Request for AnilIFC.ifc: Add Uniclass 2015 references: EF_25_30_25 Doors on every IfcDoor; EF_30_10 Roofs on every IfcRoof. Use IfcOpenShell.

First a look at what the model holds.

```python
import ifcopenshell

model = ifcopenshell.open("AnilIFC.ifc")
print(model.schema)
print("classifications:", [c.Name for c in model.by_type("IfcClassification")])
for ifc_class in ("IfcDoor", "IfcRoof", "IfcStair", "IfcWall", "IfcWindow"):
    print(ifc_class, len(model.by_type(ifc_class)))
```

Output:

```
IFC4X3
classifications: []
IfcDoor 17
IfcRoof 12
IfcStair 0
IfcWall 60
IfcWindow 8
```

```python
import ifcopenshell
import ifcopenshell.api.classification

model = ifcopenshell.open("AnilIFC.ifc")

system = ifcopenshell.api.classification.add_classification(model, classification="Uniclass 2015")

codes = {
    "IfcDoor": ("EF_25_30_25", "Doors"),
    "IfcRoof": ("EF_30_10", "Roofs"),
}
for ifc_class, (code, name) in codes.items():
    products = model.by_type(ifc_class)
    ifcopenshell.api.classification.add_reference(
        model, products=products, classification=system, identification=code, name=name
    )
    print(code, len(products))

model.write("AnilIFC-out.ifc")
```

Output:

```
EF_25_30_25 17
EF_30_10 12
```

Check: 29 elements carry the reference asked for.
